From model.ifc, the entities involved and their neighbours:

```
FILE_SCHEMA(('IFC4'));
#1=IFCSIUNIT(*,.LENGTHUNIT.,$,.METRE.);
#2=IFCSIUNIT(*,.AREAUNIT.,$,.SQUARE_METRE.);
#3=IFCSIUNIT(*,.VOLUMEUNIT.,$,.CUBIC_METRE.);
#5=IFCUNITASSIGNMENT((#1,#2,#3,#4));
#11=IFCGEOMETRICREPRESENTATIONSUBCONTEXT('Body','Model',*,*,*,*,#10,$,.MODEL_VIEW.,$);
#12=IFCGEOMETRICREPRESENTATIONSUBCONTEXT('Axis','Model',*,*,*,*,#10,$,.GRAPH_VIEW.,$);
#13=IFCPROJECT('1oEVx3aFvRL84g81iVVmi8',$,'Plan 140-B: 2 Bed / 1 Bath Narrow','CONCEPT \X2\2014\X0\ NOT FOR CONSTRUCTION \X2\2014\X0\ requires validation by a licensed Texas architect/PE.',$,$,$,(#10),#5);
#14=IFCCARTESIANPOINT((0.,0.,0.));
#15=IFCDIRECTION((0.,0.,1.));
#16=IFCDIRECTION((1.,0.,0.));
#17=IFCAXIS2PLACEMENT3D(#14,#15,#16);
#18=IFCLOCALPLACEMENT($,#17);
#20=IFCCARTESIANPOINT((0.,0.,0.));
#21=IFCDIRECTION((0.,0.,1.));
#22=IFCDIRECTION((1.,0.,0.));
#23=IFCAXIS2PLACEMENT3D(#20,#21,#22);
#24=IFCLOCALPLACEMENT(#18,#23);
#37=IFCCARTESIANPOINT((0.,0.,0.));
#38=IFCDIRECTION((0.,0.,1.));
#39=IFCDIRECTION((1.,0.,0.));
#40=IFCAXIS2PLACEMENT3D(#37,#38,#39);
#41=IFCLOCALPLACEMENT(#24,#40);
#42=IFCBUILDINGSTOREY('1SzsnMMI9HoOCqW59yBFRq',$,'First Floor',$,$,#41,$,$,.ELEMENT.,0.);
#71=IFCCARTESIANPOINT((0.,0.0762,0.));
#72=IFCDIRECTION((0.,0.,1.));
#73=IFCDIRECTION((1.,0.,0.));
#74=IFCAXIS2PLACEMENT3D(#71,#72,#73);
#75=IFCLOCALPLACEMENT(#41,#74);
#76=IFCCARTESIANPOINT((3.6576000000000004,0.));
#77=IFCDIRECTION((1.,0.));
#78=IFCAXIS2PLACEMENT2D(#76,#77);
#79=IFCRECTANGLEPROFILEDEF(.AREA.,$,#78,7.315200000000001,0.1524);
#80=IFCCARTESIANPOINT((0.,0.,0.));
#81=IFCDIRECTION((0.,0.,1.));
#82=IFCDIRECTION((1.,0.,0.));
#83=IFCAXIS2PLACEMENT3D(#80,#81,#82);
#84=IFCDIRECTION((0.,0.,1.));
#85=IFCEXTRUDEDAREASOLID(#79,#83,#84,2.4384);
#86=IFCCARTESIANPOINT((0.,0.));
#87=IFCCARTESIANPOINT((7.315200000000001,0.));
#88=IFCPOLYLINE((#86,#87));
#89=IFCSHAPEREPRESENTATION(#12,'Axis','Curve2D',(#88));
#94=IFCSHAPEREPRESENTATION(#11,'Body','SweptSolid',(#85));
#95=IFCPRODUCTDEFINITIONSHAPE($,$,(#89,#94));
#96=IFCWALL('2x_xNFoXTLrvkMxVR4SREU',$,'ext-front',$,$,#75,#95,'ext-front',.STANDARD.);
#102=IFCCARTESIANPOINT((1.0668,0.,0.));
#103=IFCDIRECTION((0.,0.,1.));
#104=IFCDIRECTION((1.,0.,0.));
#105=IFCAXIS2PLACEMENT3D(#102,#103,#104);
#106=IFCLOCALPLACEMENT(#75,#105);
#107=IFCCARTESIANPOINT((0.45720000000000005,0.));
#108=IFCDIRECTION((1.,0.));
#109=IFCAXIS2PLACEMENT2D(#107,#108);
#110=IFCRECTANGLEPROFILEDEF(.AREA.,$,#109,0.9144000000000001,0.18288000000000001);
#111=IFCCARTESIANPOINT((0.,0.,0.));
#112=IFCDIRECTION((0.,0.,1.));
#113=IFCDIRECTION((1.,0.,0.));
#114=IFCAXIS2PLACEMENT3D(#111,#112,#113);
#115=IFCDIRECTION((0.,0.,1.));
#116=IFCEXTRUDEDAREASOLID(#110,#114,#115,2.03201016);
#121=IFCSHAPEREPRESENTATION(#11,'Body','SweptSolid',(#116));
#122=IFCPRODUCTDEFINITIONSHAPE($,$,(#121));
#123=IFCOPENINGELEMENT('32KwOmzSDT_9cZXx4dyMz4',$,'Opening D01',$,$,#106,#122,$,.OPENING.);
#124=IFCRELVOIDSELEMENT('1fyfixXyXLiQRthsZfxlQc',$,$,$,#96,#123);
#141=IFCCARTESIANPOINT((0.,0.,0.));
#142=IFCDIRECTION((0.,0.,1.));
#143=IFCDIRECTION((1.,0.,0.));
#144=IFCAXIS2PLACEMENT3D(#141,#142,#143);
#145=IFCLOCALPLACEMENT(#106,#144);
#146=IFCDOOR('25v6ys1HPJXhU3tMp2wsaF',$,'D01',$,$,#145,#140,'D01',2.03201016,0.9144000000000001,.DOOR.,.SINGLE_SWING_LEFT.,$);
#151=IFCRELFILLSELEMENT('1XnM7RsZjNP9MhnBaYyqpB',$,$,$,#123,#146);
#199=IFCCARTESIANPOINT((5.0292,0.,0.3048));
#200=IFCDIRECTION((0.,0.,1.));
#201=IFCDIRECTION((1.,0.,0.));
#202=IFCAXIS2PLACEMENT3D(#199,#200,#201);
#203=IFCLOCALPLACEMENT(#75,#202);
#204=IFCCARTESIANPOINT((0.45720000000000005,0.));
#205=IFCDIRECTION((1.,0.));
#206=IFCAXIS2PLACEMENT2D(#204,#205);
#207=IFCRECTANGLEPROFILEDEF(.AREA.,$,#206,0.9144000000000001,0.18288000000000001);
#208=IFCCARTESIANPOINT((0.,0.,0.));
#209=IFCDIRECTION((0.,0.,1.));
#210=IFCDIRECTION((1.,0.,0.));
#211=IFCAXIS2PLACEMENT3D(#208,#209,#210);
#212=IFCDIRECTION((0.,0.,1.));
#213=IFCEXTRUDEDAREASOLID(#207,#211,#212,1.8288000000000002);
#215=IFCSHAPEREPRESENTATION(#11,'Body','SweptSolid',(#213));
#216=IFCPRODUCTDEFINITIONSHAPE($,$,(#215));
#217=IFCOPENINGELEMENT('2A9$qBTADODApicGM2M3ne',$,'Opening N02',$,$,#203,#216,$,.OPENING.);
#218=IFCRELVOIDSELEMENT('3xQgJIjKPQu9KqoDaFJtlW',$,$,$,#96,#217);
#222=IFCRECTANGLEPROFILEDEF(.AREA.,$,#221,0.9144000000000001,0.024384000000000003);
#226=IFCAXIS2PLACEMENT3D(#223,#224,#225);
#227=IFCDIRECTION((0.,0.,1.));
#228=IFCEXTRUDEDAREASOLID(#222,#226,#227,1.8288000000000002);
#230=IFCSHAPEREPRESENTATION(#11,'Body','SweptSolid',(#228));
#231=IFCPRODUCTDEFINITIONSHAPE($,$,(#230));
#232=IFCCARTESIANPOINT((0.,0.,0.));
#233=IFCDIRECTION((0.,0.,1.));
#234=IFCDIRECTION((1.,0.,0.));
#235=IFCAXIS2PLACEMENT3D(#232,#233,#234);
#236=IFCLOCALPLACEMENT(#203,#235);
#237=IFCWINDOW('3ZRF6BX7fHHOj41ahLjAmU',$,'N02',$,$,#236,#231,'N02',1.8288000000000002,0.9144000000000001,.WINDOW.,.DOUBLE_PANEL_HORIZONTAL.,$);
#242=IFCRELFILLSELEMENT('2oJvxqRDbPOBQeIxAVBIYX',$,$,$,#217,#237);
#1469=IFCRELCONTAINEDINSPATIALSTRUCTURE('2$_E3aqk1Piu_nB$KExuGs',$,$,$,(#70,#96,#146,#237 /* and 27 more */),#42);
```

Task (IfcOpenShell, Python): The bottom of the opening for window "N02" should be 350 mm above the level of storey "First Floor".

```python
import numpy as np
import ifcopenshell
import ifcopenshell.api.geometry
import ifcopenshell.geom
import ifcopenshell.util.element
import ifcopenshell.util.placement
import ifcopenshell.util.shape
import ifcopenshell.util.unit

model = ifcopenshell.open("model.ifc")
unit_scale = ifcopenshell.util.unit.calculate_unit_scale(model)

window = model.by_guid("3ZRF6BX7fHHOj41ahLjAmU")
opening = window.FillsVoids[0].RelatingOpeningElement
storey = ifcopenshell.util.element.get_container(window, ifc_class="IfcBuildingStorey")
level = ifcopenshell.util.placement.get_local_placement(storey.ObjectPlacement)[2, 3]

# The opening's origin need not be at the sill, so measure its lowest point.
shape = ifcopenshell.geom.create_shape(ifcopenshell.geom.settings(), opening)
bottom = ifcopenshell.util.shape.get_shape_bottom_elevation(shape, shape.geometry) / unit_scale
dz = level + 0.35 - bottom

shift = np.array([0.0, 0.0, dz])
# The window is placed relative to its opening, so it follows when the opening moves.
matrix = ifcopenshell.util.placement.get_local_placement(opening.ObjectPlacement)
matrix[:3, 3] += shift
ifcopenshell.api.geometry.edit_object_placement(
    model, product=opening, matrix=matrix, is_si=False, should_transform_children=True
)

print(f"moved by {dz * unit_scale:+.3f} m")

model.write("model-out.ifc")
```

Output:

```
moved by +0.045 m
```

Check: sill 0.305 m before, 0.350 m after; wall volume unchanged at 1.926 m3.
